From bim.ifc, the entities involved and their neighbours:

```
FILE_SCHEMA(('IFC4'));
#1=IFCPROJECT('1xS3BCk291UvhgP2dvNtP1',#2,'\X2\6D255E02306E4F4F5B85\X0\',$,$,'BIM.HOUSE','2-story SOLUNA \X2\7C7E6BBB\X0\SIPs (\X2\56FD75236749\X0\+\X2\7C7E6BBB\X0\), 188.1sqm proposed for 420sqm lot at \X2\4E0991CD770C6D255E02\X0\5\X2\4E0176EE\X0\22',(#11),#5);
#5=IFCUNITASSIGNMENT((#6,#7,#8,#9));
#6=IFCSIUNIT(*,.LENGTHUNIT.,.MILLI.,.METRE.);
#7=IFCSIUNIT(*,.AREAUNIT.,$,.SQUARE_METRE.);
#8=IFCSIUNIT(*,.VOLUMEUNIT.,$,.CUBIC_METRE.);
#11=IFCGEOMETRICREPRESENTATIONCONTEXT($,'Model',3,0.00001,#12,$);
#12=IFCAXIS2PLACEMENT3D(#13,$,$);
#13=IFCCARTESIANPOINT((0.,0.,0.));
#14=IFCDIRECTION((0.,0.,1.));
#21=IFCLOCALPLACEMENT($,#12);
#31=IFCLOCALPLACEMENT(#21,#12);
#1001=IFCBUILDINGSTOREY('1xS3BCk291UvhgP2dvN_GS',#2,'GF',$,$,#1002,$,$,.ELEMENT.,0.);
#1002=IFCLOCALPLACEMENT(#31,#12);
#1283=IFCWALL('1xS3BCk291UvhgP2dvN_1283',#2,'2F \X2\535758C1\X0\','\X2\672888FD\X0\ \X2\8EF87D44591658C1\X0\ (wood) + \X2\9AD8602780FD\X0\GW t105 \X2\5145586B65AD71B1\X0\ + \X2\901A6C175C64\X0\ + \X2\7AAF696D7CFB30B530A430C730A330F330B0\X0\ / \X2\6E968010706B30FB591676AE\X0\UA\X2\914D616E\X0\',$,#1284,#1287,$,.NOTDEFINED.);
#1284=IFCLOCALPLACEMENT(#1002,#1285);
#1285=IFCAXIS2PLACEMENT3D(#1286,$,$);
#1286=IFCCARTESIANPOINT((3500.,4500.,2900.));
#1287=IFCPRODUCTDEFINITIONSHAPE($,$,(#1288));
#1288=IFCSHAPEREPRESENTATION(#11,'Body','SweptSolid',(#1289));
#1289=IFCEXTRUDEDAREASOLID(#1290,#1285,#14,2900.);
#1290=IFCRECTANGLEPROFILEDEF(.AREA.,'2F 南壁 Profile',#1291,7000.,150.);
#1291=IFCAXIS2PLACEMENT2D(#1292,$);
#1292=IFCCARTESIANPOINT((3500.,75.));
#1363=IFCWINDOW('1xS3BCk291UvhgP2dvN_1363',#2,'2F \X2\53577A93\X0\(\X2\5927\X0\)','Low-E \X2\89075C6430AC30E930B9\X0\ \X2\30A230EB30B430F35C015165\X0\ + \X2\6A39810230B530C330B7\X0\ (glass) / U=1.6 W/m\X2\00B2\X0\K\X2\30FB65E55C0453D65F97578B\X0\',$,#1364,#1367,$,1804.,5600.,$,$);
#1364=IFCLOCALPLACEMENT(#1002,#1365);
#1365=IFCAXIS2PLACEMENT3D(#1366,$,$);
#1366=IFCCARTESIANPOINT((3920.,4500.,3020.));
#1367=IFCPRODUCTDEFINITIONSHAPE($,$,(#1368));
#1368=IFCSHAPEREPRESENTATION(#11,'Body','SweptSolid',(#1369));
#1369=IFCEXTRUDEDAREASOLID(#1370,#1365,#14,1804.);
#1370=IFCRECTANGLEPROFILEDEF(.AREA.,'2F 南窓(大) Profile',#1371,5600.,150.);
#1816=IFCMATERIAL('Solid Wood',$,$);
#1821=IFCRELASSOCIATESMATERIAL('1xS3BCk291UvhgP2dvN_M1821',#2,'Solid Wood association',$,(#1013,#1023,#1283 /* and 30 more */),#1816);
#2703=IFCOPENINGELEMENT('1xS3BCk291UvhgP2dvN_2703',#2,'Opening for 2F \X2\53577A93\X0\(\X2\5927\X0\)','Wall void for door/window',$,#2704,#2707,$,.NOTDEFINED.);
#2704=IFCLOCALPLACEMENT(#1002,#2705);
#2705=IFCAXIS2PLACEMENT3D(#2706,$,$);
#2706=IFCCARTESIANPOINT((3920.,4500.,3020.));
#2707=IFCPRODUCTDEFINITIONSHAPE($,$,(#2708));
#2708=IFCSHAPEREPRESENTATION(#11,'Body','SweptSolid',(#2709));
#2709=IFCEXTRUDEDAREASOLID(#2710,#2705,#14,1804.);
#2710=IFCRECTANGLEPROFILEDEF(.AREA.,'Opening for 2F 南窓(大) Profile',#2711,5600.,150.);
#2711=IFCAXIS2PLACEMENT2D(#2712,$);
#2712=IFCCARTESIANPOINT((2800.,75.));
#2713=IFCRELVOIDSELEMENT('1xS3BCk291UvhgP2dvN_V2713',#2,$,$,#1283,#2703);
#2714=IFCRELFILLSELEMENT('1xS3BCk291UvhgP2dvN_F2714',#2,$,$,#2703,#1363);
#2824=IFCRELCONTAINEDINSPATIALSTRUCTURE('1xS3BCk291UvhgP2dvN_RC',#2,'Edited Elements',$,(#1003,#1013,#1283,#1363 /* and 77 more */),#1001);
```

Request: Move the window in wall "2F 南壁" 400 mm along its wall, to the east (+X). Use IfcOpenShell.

```python
import ifcopenshell
import ifcopenshell.api.geometry
import ifcopenshell.util.placement

model = ifcopenshell.open("bim.ifc")

window = model.by_guid("1xS3BCk291UvhgP2dvN_1363")
opening = window.FillsVoids[0].RelatingOpeningElement
wall = opening.VoidsElements[0].RelatingBuildingElement

wall_matrix = ifcopenshell.util.placement.get_local_placement(wall.ObjectPlacement)
shift = wall_matrix[:3, 0] * 400.0
before = ifcopenshell.util.placement.get_local_placement(window.ObjectPlacement)[:3, 3].copy()

# The window is not placed relative to its opening, so move both.
for product in (opening, window):
    matrix = ifcopenshell.util.placement.get_local_placement(product.ObjectPlacement)
    matrix[:3, 3] += shift
    ifcopenshell.api.geometry.edit_object_placement(model, product=product, matrix=matrix, is_si=False)

after = ifcopenshell.util.placement.get_local_placement(window.ObjectPlacement)[:3, 3]
print("window moved by", (after - before).round(3) + 0.0)

model.write("bim-out.ifc")
```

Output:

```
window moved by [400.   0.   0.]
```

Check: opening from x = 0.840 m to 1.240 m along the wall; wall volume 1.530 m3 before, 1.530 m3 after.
